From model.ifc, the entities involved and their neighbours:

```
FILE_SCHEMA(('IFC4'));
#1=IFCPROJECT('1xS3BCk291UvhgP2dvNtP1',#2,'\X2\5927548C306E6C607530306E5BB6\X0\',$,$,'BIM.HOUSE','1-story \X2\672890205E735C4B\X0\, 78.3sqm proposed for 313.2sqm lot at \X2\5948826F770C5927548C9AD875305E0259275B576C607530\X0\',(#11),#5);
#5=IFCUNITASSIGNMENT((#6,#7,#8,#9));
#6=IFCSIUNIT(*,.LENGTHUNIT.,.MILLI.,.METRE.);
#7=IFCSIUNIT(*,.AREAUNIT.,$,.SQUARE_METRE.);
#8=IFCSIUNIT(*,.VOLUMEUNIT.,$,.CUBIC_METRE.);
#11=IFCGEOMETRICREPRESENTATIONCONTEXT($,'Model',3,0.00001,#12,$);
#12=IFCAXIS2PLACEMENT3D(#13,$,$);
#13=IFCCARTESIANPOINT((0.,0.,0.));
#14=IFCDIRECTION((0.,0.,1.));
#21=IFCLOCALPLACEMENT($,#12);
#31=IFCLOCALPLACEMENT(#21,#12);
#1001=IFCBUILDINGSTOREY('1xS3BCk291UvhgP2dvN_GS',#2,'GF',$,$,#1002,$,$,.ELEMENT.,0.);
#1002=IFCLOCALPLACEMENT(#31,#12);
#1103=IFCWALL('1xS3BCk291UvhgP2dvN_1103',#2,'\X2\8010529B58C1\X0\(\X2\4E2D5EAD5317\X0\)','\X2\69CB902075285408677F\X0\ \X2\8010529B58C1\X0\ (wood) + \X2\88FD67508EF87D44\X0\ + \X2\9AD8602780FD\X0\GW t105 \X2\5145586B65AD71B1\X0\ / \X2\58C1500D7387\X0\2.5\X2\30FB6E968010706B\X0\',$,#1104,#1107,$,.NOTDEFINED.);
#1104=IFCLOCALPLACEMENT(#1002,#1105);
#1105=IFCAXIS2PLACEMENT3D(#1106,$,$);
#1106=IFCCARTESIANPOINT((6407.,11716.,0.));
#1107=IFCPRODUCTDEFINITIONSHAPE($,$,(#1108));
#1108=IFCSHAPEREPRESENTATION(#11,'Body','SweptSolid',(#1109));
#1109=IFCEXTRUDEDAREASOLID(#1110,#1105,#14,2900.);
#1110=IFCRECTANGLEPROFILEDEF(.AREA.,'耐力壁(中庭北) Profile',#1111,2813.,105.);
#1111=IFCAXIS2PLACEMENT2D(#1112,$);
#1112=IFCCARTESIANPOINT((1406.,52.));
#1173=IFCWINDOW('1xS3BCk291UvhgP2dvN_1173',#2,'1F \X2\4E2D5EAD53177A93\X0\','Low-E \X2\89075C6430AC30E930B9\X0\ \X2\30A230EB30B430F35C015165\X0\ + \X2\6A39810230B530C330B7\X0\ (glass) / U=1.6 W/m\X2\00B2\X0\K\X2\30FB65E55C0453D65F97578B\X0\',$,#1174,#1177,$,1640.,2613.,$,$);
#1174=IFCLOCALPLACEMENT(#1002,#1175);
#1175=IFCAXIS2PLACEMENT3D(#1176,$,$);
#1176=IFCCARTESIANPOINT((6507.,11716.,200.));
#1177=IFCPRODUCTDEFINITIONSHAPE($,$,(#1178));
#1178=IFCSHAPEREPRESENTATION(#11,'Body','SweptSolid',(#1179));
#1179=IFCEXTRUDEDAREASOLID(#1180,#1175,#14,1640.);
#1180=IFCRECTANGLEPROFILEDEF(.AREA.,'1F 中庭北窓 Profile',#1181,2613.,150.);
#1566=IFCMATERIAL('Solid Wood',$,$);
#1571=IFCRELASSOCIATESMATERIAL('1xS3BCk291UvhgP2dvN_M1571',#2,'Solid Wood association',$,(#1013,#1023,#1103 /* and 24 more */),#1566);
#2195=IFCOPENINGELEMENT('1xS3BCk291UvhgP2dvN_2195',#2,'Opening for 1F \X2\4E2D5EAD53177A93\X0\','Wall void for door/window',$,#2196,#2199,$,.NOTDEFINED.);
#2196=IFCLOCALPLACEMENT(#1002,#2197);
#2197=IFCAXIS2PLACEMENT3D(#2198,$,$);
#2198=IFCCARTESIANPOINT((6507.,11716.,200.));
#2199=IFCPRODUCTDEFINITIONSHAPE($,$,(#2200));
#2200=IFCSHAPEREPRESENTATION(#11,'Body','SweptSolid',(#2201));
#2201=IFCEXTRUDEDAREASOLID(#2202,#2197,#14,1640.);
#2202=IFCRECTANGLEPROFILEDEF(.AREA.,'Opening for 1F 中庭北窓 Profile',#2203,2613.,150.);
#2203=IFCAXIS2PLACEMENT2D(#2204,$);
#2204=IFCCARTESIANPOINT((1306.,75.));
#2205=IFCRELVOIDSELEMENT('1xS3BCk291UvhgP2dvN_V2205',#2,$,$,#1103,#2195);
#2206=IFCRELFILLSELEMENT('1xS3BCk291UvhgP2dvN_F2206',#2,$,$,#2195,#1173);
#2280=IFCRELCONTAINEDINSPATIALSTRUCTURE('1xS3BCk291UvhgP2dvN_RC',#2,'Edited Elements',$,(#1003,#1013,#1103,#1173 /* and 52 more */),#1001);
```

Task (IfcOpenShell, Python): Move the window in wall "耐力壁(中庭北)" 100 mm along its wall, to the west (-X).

```python
import ifcopenshell
import ifcopenshell.api.geometry
import ifcopenshell.util.placement
import ifcopenshell.util.unit

model = ifcopenshell.open("model.ifc")
unit_scale = ifcopenshell.util.unit.calculate_unit_scale(model)

window = model.by_guid("1xS3BCk291UvhgP2dvN_1173")
opening = window.FillsVoids[0].RelatingOpeningElement
wall = opening.VoidsElements[0].RelatingBuildingElement

wall_matrix = ifcopenshell.util.placement.get_local_placement(wall.ObjectPlacement)
shift = wall_matrix[:3, 0] * -0.1 / unit_scale
before = ifcopenshell.util.placement.get_local_placement(window.ObjectPlacement)[:3, 3].copy()

# The window is not placed relative to its opening, so move both.
for product in (opening, window):
    matrix = ifcopenshell.util.placement.get_local_placement(product.ObjectPlacement)
    matrix[:3, 3] += shift
    ifcopenshell.api.geometry.edit_object_placement(model, product=product, matrix=matrix, is_si=False)

after = ifcopenshell.util.placement.get_local_placement(window.ObjectPlacement)[:3, 3]
print("window moved by", (after - before).round(3) + 0.0)

model.write("model_v2.ifc")
```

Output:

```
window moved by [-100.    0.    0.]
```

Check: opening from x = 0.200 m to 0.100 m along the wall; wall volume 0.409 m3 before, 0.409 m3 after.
